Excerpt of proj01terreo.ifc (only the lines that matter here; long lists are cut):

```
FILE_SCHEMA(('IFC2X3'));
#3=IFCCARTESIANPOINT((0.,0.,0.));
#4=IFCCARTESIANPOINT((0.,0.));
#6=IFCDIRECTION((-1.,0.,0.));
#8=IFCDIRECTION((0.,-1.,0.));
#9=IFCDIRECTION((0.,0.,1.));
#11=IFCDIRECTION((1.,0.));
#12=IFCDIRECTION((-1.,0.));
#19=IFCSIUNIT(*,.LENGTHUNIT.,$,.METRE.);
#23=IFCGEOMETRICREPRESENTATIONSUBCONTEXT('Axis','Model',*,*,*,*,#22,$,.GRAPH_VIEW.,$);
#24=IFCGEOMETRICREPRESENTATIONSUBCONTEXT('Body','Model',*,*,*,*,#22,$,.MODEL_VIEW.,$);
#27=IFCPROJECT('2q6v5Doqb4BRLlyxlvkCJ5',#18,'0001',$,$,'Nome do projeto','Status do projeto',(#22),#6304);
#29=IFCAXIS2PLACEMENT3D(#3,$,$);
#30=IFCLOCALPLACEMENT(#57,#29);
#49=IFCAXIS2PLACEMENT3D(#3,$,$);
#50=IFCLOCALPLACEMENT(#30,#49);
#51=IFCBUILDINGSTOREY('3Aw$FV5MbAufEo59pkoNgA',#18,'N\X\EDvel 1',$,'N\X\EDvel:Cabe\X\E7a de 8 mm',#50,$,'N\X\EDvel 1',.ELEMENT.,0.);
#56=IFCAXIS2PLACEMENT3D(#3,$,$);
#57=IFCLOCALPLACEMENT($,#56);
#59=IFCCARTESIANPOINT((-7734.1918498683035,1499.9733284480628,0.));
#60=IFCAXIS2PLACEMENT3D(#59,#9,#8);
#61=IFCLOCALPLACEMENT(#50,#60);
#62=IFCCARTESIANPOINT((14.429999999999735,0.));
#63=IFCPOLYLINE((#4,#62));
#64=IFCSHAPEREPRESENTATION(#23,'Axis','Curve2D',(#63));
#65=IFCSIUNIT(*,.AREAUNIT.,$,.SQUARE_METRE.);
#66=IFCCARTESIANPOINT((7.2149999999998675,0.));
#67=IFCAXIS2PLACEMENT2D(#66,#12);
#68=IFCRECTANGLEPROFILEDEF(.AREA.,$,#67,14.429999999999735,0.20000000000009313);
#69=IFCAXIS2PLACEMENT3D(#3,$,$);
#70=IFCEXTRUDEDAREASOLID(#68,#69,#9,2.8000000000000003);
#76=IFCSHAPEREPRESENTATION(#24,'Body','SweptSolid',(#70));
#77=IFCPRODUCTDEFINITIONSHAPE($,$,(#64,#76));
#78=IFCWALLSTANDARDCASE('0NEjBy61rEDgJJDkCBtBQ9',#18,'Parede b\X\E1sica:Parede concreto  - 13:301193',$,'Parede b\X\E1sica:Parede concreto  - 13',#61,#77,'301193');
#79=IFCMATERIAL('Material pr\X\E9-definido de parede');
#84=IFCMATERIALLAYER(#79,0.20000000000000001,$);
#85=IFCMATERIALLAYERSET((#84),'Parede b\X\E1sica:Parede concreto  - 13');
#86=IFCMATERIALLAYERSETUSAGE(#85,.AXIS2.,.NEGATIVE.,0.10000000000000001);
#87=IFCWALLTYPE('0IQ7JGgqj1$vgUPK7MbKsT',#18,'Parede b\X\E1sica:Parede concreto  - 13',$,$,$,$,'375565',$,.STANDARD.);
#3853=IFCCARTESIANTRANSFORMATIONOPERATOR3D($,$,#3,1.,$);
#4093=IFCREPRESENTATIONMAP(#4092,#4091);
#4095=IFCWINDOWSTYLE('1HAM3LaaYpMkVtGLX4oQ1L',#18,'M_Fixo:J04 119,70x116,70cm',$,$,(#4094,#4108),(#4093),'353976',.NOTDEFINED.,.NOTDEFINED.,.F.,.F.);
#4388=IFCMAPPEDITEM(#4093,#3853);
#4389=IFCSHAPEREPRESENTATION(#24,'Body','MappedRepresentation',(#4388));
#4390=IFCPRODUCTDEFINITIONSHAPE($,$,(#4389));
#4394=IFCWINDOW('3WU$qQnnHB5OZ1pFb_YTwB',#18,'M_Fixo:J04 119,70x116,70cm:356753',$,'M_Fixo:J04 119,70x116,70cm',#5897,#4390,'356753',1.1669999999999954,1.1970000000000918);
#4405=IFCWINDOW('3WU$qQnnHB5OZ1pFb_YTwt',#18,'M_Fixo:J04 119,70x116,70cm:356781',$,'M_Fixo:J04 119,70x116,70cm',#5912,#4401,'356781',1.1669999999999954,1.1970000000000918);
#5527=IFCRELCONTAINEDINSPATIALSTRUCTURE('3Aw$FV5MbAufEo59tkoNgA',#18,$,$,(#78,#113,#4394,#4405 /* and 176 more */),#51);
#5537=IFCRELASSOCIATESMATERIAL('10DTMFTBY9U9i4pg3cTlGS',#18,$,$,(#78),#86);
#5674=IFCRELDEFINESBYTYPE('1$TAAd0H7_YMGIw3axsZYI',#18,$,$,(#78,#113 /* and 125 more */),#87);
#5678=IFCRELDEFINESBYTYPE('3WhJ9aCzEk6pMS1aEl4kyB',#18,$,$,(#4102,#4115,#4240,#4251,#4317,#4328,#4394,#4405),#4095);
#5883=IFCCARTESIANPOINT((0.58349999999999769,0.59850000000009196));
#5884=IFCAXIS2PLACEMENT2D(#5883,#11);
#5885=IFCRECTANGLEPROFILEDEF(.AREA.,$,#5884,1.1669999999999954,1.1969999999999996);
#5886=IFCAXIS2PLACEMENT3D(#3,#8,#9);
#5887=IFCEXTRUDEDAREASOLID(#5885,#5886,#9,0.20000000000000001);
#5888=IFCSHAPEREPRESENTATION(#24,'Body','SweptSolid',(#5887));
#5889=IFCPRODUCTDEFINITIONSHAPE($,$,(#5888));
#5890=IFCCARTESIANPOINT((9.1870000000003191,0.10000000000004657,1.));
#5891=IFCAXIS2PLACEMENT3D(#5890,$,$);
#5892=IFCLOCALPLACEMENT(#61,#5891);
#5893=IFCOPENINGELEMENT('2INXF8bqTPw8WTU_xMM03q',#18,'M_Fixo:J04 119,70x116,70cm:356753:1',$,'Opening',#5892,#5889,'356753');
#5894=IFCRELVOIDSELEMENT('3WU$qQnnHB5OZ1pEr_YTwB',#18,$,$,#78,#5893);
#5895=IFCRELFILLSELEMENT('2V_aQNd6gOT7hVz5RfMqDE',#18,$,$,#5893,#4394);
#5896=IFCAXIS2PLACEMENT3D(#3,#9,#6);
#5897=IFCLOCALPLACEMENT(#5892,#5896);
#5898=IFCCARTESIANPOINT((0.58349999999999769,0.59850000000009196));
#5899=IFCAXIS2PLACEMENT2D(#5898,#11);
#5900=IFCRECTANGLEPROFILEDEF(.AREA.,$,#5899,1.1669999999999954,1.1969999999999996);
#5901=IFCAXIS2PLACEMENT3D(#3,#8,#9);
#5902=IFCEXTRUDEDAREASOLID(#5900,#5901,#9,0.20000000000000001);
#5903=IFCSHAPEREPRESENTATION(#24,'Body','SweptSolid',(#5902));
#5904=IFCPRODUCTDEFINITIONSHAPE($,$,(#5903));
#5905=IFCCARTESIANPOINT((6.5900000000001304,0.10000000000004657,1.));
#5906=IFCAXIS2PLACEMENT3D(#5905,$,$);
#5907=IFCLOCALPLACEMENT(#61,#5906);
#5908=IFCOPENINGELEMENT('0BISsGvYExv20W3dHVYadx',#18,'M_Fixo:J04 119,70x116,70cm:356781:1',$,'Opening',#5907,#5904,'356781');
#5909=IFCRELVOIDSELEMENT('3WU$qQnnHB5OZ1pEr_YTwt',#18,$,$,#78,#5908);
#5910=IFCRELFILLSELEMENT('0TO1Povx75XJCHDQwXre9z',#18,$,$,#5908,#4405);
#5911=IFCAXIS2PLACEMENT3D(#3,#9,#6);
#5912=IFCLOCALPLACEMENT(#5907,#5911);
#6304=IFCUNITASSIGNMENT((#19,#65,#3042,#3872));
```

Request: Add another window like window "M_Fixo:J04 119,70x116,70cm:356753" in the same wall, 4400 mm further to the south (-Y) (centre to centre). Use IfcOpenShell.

```python
import ifcopenshell
import ifcopenshell.api.feature
import ifcopenshell.api.geometry
import ifcopenshell.api.root
import ifcopenshell.geom
import ifcopenshell.util.element
import ifcopenshell.util.placement
import ifcopenshell.util.shape
import ifcopenshell.util.unit

model = ifcopenshell.open("proj01terreo.ifc")
unit_scale = ifcopenshell.util.unit.calculate_unit_scale(model)
settings = ifcopenshell.geom.settings()


def volume(element):
    """Net volume in cubic metres, openings subtracted."""
    shape = ifcopenshell.geom.create_shape(settings, element)
    return ifcopenshell.util.shape.get_volume(shape.geometry)


def reuse_history(source, copy):
    """copy_class also copies each property set's owner history, people and application; keep the originals."""
    for rel in copy.IsDefinedBy:
        if rel.is_a("IfcRelDefinesByProperties") and (history := rel.RelatingPropertyDefinition.OwnerHistory):
            rel.RelatingPropertyDefinition.OwnerHistory = source.OwnerHistory
            ifcopenshell.util.element.remove_deep2(model, history)


window = model.by_id(4394)
opening = window.FillsVoids[0].RelatingOpeningElement
wall = opening.VoidsElements[0].RelatingBuildingElement
before = volume(wall)
shift = ifcopenshell.util.placement.get_local_placement(wall.ObjectPlacement)[:3, 0] * 4.4 / unit_scale

# copy_class copies the void relationship, type, container and properties, but no geometry.
new_opening = ifcopenshell.api.root.copy_class(model, product=opening)
new_opening.Representation = ifcopenshell.util.element.copy_deep(
    model, opening.Representation, exclude=["IfcGeometricRepresentationContext", "IfcRepresentationMap"]
)
new_opening.Name = "M_Fixo:J04 119,70x116,70cm"
new_opening.Tag = None
new_window = ifcopenshell.api.root.copy_class(model, product=window)
new_window.Representation = ifcopenshell.util.element.copy_deep(
    model, window.Representation, exclude=["IfcGeometricRepresentationContext", "IfcRepresentationMap"]
)
new_window.Name = "M_Fixo:J04 119,70x116,70cm"
new_window.Tag = None
reuse_history(window, new_window)
fills = ifcopenshell.api.feature.add_filling(model, opening=new_opening, element=new_window)
fills.OwnerHistory = new_window.OwnerHistory  # required in IFC2X3

for old, new in ((opening, new_opening), (window, new_window)):
    matrix = ifcopenshell.util.placement.get_local_placement(old.ObjectPlacement)
    matrix[:3, 3] += shift
    ifcopenshell.api.geometry.edit_object_placement(model, product=new, matrix=matrix, is_si=False)

after = volume(wall)

print(f"wall volume {before:.3f} -> {after:.3f} m3")

model.write("proj01terreo_edited.ifc")
```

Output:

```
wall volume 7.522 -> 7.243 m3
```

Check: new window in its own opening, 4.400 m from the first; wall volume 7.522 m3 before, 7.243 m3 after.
